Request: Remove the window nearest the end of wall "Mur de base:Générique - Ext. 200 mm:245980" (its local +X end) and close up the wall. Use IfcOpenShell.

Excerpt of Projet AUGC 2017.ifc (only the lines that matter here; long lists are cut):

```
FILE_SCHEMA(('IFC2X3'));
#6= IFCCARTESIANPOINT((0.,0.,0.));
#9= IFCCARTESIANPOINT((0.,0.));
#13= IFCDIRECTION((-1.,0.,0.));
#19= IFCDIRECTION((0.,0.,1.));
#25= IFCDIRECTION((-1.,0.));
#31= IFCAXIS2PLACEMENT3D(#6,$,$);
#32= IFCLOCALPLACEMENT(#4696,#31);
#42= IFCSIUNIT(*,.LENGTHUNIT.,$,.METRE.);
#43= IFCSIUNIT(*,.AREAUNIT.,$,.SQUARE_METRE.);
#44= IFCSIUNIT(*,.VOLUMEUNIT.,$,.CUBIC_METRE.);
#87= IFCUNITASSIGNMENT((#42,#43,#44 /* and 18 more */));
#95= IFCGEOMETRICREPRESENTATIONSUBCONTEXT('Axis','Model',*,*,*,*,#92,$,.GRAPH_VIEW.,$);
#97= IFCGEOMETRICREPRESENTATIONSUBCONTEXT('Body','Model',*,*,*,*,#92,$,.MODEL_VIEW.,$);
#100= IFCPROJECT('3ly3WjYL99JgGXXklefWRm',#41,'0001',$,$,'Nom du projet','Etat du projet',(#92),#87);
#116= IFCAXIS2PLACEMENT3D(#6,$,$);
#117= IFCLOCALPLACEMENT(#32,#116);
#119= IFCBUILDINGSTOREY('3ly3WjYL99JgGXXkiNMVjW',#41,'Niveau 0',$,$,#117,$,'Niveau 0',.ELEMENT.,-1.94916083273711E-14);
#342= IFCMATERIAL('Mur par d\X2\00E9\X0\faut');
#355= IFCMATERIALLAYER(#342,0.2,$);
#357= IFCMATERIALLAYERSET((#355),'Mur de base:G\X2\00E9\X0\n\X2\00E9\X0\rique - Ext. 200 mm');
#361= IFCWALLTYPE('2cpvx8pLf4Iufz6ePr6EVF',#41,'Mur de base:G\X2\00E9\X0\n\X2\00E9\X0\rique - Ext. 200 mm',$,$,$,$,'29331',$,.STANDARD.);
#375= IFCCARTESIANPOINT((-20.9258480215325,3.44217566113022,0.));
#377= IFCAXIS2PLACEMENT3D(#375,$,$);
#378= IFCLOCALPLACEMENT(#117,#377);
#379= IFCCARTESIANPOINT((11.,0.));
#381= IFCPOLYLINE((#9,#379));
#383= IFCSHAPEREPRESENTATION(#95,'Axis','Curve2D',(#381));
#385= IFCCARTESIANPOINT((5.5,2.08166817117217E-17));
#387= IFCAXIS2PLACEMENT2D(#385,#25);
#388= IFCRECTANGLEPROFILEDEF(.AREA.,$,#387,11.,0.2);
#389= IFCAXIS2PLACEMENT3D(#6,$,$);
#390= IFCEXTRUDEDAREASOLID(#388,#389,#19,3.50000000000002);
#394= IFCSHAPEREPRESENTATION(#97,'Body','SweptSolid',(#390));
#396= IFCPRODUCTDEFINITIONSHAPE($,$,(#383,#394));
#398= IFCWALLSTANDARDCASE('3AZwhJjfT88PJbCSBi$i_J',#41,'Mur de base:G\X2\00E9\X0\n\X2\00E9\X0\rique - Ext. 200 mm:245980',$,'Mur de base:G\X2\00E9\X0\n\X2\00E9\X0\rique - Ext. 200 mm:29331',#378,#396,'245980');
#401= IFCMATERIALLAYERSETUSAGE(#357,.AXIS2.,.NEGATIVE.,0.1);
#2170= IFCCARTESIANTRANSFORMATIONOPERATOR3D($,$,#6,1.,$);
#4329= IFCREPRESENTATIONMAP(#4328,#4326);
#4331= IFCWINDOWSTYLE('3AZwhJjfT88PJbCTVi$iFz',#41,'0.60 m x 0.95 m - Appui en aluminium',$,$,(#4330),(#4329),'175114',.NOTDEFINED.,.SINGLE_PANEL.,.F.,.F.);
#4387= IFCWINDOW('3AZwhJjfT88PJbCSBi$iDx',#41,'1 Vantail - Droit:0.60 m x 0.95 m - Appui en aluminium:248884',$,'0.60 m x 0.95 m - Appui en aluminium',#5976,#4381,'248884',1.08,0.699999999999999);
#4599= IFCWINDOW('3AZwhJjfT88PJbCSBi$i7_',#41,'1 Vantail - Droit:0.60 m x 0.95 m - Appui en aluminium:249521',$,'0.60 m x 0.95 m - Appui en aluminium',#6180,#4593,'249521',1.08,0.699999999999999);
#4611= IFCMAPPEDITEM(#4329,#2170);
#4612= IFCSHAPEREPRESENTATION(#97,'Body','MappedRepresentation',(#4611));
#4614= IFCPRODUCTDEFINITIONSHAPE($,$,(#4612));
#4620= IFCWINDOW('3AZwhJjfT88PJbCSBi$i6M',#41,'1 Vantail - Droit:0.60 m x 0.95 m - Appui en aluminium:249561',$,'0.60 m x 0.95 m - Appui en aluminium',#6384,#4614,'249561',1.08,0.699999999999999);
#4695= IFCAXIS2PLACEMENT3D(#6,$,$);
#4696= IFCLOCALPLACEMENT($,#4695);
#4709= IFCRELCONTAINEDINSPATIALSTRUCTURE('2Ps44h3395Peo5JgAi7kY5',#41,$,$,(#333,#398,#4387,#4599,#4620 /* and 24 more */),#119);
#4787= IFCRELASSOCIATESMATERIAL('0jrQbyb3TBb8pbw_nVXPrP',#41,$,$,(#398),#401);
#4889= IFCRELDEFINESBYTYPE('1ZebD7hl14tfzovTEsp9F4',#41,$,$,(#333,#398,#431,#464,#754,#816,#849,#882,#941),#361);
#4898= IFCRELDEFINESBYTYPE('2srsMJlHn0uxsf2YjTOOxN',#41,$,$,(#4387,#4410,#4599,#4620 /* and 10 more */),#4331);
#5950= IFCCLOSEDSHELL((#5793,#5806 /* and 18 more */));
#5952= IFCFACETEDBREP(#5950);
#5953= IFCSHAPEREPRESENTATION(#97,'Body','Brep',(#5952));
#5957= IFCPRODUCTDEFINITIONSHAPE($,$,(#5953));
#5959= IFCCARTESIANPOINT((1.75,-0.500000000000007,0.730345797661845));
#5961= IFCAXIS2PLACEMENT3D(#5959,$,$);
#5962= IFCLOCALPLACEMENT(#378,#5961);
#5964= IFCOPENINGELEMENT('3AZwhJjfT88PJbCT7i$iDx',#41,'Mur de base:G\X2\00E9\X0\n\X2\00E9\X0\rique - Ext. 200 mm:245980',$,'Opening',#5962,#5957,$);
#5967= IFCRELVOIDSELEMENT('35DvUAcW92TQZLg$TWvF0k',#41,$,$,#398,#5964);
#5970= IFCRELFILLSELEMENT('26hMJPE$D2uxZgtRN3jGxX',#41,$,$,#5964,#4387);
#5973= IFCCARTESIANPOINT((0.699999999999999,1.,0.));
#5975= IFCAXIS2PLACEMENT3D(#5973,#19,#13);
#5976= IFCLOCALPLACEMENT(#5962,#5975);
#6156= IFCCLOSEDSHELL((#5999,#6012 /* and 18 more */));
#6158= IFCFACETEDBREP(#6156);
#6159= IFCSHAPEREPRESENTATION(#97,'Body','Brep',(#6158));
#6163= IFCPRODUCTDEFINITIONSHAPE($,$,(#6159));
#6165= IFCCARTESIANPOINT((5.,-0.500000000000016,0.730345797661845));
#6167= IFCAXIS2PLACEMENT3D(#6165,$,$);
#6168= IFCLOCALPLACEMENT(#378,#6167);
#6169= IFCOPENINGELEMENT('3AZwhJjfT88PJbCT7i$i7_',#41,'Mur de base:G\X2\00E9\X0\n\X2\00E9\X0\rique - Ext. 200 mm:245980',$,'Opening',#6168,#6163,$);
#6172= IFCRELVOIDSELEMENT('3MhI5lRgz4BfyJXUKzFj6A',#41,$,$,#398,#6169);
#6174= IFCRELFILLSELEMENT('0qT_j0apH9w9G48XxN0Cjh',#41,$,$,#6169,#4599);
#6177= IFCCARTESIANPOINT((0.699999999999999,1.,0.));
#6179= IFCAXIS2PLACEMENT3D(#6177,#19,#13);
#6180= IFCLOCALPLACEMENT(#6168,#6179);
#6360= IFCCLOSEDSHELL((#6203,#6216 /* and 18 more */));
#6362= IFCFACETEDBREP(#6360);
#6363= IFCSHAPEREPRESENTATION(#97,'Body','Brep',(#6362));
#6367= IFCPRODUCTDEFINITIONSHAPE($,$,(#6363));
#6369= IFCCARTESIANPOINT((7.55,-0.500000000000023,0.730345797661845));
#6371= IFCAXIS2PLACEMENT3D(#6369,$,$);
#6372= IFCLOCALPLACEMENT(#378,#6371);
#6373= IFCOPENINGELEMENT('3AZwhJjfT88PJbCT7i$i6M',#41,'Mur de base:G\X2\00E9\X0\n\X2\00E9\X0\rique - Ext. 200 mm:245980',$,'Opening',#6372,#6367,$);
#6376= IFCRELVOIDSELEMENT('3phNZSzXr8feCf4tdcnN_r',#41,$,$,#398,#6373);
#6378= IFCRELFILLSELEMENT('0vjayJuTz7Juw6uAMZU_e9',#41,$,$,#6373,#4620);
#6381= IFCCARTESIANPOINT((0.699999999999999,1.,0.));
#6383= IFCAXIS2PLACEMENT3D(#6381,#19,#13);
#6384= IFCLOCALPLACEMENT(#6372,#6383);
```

```python
import ifcopenshell
import ifcopenshell.api.feature
import ifcopenshell.api.root
import ifcopenshell.geom
import ifcopenshell.util.shape

model = ifcopenshell.open("Projet AUGC 2017.ifc")
settings = ifcopenshell.geom.settings()


def volume(element):
    """Net volume in cubic metres, openings subtracted."""
    shape = ifcopenshell.geom.create_shape(settings, element)
    return ifcopenshell.util.shape.get_volume(shape.geometry)


window = model.by_guid("3AZwhJjfT88PJbCSBi$i6M")
opening = window.FillsVoids[0].RelatingOpeningElement
wall = opening.VoidsElements[0].RelatingBuildingElement
before = volume(wall)

ifcopenshell.api.root.remove_product(model, product=window)
ifcopenshell.api.feature.remove_feature(model, feature=opening)

after = volume(wall)

print(f"wall volume {before:.3f} -> {after:.3f} m3")

model.write("Projet AUGC 2017-out.ifc")
```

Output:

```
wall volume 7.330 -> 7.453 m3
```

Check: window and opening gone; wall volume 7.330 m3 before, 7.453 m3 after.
